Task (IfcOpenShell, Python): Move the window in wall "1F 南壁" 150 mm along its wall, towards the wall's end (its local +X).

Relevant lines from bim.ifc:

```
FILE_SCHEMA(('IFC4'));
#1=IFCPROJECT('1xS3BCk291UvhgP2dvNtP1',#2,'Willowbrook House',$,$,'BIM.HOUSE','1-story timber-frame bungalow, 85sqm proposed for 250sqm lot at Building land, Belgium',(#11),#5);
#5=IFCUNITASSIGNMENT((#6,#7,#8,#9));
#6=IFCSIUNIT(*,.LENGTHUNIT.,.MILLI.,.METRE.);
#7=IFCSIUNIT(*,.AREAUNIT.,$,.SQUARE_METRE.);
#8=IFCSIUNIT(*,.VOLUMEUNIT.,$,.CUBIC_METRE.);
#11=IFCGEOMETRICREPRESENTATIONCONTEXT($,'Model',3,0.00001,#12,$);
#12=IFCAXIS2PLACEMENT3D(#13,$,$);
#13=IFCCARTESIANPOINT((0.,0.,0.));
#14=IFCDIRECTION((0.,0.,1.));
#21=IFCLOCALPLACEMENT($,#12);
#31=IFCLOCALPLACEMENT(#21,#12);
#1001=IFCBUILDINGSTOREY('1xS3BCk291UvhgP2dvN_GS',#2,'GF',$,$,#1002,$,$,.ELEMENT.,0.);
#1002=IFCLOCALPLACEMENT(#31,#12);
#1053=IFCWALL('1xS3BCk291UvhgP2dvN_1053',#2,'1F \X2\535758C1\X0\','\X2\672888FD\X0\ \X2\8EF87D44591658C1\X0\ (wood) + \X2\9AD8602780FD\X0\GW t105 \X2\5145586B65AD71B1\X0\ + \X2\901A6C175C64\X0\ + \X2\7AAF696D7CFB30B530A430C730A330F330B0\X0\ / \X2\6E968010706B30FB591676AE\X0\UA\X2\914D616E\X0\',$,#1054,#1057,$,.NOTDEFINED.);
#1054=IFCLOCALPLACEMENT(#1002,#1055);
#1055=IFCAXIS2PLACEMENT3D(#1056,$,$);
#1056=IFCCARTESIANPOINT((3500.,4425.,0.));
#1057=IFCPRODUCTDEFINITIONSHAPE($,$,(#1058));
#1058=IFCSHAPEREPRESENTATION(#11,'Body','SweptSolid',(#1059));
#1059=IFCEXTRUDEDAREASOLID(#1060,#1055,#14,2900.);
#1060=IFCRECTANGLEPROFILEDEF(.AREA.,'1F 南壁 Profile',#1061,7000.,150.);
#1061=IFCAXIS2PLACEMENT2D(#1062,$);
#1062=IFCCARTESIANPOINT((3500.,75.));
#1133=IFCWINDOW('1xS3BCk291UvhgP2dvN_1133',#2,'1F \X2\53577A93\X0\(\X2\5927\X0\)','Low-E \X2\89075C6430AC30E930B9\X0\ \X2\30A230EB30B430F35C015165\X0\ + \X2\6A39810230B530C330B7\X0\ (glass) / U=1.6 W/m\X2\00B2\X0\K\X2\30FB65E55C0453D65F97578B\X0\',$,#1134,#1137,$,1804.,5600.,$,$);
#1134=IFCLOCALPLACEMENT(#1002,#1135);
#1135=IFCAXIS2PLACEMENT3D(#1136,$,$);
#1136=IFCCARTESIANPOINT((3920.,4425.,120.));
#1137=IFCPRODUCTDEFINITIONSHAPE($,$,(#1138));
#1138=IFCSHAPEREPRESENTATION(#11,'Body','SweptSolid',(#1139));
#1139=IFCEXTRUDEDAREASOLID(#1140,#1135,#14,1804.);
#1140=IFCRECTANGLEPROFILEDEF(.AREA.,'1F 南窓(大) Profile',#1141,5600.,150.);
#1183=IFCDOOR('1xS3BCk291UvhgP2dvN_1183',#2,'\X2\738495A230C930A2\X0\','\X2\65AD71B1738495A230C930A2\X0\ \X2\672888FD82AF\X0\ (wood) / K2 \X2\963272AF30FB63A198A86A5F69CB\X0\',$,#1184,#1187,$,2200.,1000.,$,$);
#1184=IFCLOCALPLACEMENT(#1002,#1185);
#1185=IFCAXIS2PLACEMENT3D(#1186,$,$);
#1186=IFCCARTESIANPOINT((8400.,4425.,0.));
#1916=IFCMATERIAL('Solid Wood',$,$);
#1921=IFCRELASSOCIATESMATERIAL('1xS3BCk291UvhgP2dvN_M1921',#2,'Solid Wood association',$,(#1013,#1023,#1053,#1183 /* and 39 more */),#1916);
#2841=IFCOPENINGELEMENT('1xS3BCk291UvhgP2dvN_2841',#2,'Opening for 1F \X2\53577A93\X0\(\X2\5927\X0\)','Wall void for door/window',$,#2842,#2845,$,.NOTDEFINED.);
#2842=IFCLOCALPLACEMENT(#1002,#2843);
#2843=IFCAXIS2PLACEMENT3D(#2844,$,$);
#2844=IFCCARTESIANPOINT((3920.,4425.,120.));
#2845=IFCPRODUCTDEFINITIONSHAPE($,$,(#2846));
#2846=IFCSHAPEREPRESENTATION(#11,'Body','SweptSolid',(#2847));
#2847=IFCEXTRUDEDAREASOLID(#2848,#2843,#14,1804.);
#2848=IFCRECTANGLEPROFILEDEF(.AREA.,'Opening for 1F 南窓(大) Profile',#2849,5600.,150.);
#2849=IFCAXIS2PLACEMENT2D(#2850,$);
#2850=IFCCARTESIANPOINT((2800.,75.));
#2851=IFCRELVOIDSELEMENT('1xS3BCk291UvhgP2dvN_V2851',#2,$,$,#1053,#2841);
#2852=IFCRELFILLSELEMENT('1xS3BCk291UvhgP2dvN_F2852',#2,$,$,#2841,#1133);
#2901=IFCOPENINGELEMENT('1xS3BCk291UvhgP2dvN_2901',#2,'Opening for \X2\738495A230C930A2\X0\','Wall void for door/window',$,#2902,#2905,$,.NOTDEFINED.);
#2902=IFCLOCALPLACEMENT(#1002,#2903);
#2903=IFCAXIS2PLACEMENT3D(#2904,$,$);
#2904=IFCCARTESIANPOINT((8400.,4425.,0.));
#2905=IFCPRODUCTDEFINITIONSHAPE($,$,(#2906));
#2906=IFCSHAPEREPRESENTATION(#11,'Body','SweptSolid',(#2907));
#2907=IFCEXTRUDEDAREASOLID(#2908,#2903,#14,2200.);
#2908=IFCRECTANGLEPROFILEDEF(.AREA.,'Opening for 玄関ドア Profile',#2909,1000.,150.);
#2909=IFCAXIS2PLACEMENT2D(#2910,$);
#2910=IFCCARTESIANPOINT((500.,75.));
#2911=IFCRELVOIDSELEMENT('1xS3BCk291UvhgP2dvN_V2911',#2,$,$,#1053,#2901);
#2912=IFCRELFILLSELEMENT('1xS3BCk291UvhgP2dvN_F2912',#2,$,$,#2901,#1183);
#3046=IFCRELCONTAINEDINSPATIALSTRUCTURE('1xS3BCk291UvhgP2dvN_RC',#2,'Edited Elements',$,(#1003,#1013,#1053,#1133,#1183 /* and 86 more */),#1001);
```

```python
import ifcopenshell
import ifcopenshell.api.geometry
import ifcopenshell.util.placement

model = ifcopenshell.open("bim.ifc")

window = model.by_guid("1xS3BCk291UvhgP2dvN_1133")
opening = window.FillsVoids[0].RelatingOpeningElement
wall = opening.VoidsElements[0].RelatingBuildingElement

wall_matrix = ifcopenshell.util.placement.get_local_placement(wall.ObjectPlacement)
shift = wall_matrix[:3, 0] * 150.0
before = ifcopenshell.util.placement.get_local_placement(window.ObjectPlacement)[:3, 3].copy()

# The window is not placed relative to its opening, so move both.
for product in (opening, window):
    matrix = ifcopenshell.util.placement.get_local_placement(product.ObjectPlacement)
    matrix[:3, 3] += shift
    ifcopenshell.api.geometry.edit_object_placement(model, product=product, matrix=matrix, is_si=False)

after = ifcopenshell.util.placement.get_local_placement(window.ObjectPlacement)[:3, 3]
print("window moved by", (after - before).round(3) + 0.0)

model.write("bim_rev.ifc")
```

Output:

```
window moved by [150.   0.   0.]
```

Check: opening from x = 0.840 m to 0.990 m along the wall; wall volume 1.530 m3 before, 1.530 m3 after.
